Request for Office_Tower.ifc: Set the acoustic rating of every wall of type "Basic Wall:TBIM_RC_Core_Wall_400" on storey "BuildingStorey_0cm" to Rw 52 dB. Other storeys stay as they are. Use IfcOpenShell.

First a look at what the model holds.

```python
import ifcopenshell
import ifcopenshell.util.element

model = ifcopenshell.open("Office_Tower.ifc")
print(model.schema)
storey = next(s for s in model.by_type("IfcBuildingStorey") if s.Name == "BuildingStorey_0cm")
walls = [e for e in ifcopenshell.util.element.get_decomposition(storey) if e.is_a("IfcWall")]
seen = {}
for e in walls:
    element_type = ifcopenshell.util.element.get_type(e)
    key = (element_type.Name if element_type != e and element_type else None, ifcopenshell.util.element.get_pset(e, "Pset_WallCommon", "AcousticRating"))
    seen[key] = seen.get(key, 0) + 1
for (name, value), count in sorted(seen.items(), key=str):
    print(count, "x", name, "|", value)
```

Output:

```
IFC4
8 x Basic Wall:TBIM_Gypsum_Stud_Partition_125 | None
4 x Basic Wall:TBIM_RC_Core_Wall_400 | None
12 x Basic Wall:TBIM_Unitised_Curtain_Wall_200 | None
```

```python
import ifcopenshell
import ifcopenshell.api.pset
import ifcopenshell.util.element

model = ifcopenshell.open("Office_Tower.ifc")

storey = next(s for s in model.by_type("IfcBuildingStorey") if s.Name == "BuildingStorey_0cm")
walls = [e for e in ifcopenshell.util.element.get_decomposition(storey) if e.is_a("IfcWall")]

count = 0
for e in walls:
    element_type = ifcopenshell.util.element.get_type(e)
    if element_type in (None, e) or element_type.Name != "Basic Wall:TBIM_RC_Core_Wall_400":
        continue
    # add_pset returns the element's existing set when there is one.
    pset = ifcopenshell.api.pset.add_pset(model, product=e, name="Pset_WallCommon")
    ifcopenshell.api.pset.edit_pset(model, pset=pset, properties={"AcousticRating": "Rw 52 dB"})
    count += 1

print(count, "walls updated")

model.write("Office_Tower_rev.ifc")
```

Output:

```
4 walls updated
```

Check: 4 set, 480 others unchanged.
